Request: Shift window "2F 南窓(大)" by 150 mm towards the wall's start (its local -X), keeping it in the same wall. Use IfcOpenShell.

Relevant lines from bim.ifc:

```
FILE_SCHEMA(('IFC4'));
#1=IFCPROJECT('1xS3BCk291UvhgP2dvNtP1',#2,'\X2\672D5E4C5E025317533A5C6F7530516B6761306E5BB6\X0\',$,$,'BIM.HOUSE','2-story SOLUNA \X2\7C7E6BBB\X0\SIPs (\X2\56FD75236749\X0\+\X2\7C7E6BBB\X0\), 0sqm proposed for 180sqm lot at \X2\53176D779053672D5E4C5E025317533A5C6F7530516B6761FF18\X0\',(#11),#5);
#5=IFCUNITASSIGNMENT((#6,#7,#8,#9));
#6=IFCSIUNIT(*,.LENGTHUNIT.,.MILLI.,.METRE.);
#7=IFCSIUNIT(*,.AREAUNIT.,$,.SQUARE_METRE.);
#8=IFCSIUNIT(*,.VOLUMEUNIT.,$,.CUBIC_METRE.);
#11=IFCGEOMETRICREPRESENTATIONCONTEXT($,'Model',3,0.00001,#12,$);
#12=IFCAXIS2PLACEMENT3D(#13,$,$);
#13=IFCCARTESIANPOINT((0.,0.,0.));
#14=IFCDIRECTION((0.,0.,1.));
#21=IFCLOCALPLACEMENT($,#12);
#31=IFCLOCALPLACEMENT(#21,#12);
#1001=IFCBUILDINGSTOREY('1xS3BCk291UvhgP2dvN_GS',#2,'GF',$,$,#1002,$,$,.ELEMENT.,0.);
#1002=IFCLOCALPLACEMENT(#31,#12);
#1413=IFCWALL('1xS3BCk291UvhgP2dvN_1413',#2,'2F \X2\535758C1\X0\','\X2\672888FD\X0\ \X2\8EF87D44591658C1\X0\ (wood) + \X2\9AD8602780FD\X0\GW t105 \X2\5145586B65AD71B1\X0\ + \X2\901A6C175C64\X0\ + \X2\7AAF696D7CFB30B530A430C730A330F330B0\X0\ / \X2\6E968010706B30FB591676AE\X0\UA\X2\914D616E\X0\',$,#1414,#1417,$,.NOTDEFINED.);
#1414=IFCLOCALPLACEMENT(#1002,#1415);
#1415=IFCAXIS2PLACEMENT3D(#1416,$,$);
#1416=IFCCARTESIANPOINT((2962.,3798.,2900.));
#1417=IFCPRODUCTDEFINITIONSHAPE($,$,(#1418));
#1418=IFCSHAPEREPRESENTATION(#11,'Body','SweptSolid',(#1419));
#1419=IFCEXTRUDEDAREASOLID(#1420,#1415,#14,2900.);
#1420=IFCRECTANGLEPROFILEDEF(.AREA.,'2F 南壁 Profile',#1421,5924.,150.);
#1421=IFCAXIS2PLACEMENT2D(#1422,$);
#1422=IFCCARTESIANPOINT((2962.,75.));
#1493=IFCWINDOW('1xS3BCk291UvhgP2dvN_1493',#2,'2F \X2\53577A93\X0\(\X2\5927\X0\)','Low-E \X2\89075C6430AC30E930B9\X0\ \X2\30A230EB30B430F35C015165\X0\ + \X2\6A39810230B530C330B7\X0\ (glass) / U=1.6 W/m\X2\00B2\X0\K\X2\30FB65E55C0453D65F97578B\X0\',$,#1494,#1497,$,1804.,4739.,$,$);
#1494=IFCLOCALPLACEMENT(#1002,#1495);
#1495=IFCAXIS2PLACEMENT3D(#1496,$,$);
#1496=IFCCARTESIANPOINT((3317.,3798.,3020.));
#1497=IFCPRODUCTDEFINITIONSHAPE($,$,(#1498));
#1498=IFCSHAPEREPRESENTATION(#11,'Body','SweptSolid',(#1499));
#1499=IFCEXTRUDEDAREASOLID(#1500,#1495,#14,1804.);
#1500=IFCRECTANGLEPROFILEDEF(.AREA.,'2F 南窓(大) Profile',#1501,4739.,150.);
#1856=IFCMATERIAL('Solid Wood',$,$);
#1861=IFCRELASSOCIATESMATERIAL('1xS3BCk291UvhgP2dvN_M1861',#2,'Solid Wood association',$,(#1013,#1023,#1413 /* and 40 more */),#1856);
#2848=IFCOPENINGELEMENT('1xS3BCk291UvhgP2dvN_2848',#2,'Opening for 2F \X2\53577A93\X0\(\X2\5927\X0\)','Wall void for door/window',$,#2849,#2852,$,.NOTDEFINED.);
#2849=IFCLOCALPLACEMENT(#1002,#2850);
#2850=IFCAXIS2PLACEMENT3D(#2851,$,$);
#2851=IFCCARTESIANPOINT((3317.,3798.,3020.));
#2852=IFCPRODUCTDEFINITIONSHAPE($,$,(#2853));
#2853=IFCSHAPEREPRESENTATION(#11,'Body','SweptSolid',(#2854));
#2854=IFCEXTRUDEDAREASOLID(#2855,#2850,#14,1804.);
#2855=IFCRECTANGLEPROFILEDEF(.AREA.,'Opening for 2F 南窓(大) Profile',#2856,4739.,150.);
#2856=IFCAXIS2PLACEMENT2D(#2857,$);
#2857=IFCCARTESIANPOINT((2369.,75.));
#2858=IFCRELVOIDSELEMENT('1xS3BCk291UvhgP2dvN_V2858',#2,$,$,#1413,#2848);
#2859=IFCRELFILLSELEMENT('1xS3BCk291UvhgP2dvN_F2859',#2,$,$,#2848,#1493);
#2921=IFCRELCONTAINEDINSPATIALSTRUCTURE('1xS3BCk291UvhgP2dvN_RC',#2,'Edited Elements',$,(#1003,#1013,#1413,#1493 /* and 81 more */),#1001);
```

```python
import ifcopenshell
import ifcopenshell.api.geometry
import ifcopenshell.util.placement
import ifcopenshell.util.unit

model = ifcopenshell.open("bim.ifc")
unit_scale = ifcopenshell.util.unit.calculate_unit_scale(model)

window = model.by_guid("1xS3BCk291UvhgP2dvN_1493")
opening = window.FillsVoids[0].RelatingOpeningElement
wall = opening.VoidsElements[0].RelatingBuildingElement

wall_matrix = ifcopenshell.util.placement.get_local_placement(wall.ObjectPlacement)
shift = wall_matrix[:3, 0] * -0.15 / unit_scale
before = ifcopenshell.util.placement.get_local_placement(window.ObjectPlacement)[:3, 3].copy()

# The window is not placed relative to its opening, so move both.
for product in (opening, window):
    matrix = ifcopenshell.util.placement.get_local_placement(product.ObjectPlacement)
    matrix[:3, 3] += shift
    ifcopenshell.api.geometry.edit_object_placement(model, product=product, matrix=matrix, is_si=False)

after = ifcopenshell.util.placement.get_local_placement(window.ObjectPlacement)[:3, 3]
print("window moved by", (after - before).round(3) + 0.0)

model.write("bim_updated.ifc")
```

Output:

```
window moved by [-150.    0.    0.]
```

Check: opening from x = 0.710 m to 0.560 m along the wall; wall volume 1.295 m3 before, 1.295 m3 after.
